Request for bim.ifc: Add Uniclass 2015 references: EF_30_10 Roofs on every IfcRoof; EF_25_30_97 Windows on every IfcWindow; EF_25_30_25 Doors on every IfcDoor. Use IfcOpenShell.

First a look at what the model holds.

```python
import ifcopenshell

model = ifcopenshell.open("bim.ifc")
print(model.schema)
print("classifications:", [c.Name for c in model.by_type("IfcClassification")])
for ifc_class in ("IfcDoor", "IfcRoof", "IfcStair", "IfcWall", "IfcWindow"):
    print(ifc_class, len(model.by_type(ifc_class)))
```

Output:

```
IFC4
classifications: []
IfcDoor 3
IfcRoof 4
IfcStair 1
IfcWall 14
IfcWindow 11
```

```python
import ifcopenshell
import ifcopenshell.api.classification

model = ifcopenshell.open("bim.ifc")

system = ifcopenshell.api.classification.add_classification(model, classification="Uniclass 2015")

codes = {
    "IfcRoof": ("EF_30_10", "Roofs"),
    "IfcWindow": ("EF_25_30_97", "Windows"),
    "IfcDoor": ("EF_25_30_25", "Doors"),
}
for ifc_class, (code, name) in codes.items():
    products = model.by_type(ifc_class)
    ifcopenshell.api.classification.add_reference(
        model, products=products, classification=system, identification=code, name=name
    )
    print(code, len(products))

model.write("bim-out.ifc")
```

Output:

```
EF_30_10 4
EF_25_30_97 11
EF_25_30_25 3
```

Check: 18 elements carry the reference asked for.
